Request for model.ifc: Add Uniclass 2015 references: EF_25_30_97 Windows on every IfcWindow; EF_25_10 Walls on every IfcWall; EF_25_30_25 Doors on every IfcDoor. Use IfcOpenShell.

First a look at what the model holds.

```python
import ifcopenshell

model = ifcopenshell.open("model.ifc")
print(model.schema)
print("classifications:", [c.Name for c in model.by_type("IfcClassification")])
for ifc_class in ("IfcDoor", "IfcRoof", "IfcStair", "IfcWall", "IfcWindow"):
    print(ifc_class, len(model.by_type(ifc_class)))
```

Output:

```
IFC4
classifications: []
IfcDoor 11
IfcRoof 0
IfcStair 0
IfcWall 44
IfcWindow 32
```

```python
import ifcopenshell
import ifcopenshell.api.classification

model = ifcopenshell.open("model.ifc")

system = ifcopenshell.api.classification.add_classification(model, classification="Uniclass 2015")

codes = {
    "IfcWindow": ("EF_25_30_97", "Windows"),
    "IfcWall": ("EF_25_10", "Walls"),
    "IfcDoor": ("EF_25_30_25", "Doors"),
}
for ifc_class, (code, name) in codes.items():
    products = model.by_type(ifc_class)
    ifcopenshell.api.classification.add_reference(
        model, products=products, classification=system, identification=code, name=name
    )
    print(code, len(products))

model.write("model-out.ifc")
```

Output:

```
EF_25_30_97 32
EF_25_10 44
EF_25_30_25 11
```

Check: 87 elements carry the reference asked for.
